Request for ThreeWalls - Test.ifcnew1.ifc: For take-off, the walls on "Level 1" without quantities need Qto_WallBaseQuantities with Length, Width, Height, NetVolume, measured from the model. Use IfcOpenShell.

First a look at what the model holds.

```python
import ifcopenshell
import ifcopenshell.util.element
import ifcopenshell.util.unit

model = ifcopenshell.open("ThreeWalls - Test.ifcnew1.ifc")
print(model.schema)
for unit_type in ("LENGTHUNIT", "AREAUNIT", "VOLUMEUNIT"):
    print(unit_type, ifcopenshell.util.unit.calculate_unit_scale(model, unit_type))
storey = next(s for s in model.by_type("IfcBuildingStorey") if s.Name == "Level 1")
walls = [e for e in ifcopenshell.util.element.get_decomposition(storey) if e.is_a("IfcWall")]
for e in sorted(walls, key=lambda e: e.id()):
    print(e.id(), e.is_a(), e.Name, list(ifcopenshell.util.element.get_psets(e, qtos_only=True)), sep=" | ")
```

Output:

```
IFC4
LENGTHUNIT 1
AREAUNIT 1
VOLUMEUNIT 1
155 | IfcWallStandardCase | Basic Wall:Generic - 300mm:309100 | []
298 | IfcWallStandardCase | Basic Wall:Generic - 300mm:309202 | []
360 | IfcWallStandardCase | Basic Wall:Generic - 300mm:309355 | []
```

```python
import ifcopenshell
import ifcopenshell.api.pset
import ifcopenshell.geom
import ifcopenshell.util.element
import ifcopenshell.util.shape
import ifcopenshell.util.unit

model = ifcopenshell.open("ThreeWalls - Test.ifcnew1.ifc")
unit_scale = ifcopenshell.util.unit.calculate_unit_scale(model)
volume_scale = ifcopenshell.util.unit.calculate_unit_scale(model, "VOLUMEUNIT")
settings = ifcopenshell.geom.settings()

storey = next(s for s in model.by_type("IfcBuildingStorey") if s.Name == "Level 1")
walls = [e for e in ifcopenshell.util.element.get_decomposition(storey) if e.is_a("IfcWall")]

for e in sorted(walls, key=lambda e: e.id()):
    if ifcopenshell.util.element.get_psets(e, qtos_only=True, should_inherit=False):
        continue
    # Geometry comes back in metres, in the element's own axes.
    shape = ifcopenshell.geom.create_shape(settings, e)
    values = {
        "Length": ifcopenshell.util.shape.get_x(shape.geometry) / unit_scale,
        "Width": ifcopenshell.util.shape.get_y(shape.geometry) / unit_scale,
        "Height": ifcopenshell.util.shape.get_z(shape.geometry) / unit_scale,
        "NetVolume": ifcopenshell.util.shape.get_volume(shape.geometry) / volume_scale,
    }
    qto = ifcopenshell.api.pset.add_qto(model, product=e, name="Qto_WallBaseQuantities")
    ifcopenshell.api.pset.edit_qto(model, qto=qto, properties=values)
    print(e.id(), {k: round(v, 3) for k, v in values.items()})

model.write("ThreeWalls - Test.ifcnew1_updated.ifc")
```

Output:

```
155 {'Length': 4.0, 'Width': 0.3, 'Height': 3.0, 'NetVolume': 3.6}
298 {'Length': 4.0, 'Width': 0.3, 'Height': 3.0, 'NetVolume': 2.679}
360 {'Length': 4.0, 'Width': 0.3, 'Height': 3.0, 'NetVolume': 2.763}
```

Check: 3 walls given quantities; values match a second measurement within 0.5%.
